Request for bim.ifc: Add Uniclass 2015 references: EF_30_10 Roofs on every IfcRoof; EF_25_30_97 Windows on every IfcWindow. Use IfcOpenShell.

First a look at what the model holds.

```python
import ifcopenshell

model = ifcopenshell.open("bim.ifc")
print(model.schema)
print("classifications:", [c.Name for c in model.by_type("IfcClassification")])
for ifc_class in ("IfcDoor", "IfcRoof", "IfcStair", "IfcWall", "IfcWindow"):
    print(ifc_class, len(model.by_type(ifc_class)))
```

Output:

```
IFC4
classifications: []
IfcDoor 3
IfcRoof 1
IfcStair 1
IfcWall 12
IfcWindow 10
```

```python
import ifcopenshell
import ifcopenshell.api.classification

model = ifcopenshell.open("bim.ifc")

system = ifcopenshell.api.classification.add_classification(model, classification="Uniclass 2015")

codes = {
    "IfcRoof": ("EF_30_10", "Roofs"),
    "IfcWindow": ("EF_25_30_97", "Windows"),
}
for ifc_class, (code, name) in codes.items():
    products = model.by_type(ifc_class)
    ifcopenshell.api.classification.add_reference(
        model, products=products, classification=system, identification=code, name=name
    )
    print(code, len(products))

model.write("bim-out.ifc")
```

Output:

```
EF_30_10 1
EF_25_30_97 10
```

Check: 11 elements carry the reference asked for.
